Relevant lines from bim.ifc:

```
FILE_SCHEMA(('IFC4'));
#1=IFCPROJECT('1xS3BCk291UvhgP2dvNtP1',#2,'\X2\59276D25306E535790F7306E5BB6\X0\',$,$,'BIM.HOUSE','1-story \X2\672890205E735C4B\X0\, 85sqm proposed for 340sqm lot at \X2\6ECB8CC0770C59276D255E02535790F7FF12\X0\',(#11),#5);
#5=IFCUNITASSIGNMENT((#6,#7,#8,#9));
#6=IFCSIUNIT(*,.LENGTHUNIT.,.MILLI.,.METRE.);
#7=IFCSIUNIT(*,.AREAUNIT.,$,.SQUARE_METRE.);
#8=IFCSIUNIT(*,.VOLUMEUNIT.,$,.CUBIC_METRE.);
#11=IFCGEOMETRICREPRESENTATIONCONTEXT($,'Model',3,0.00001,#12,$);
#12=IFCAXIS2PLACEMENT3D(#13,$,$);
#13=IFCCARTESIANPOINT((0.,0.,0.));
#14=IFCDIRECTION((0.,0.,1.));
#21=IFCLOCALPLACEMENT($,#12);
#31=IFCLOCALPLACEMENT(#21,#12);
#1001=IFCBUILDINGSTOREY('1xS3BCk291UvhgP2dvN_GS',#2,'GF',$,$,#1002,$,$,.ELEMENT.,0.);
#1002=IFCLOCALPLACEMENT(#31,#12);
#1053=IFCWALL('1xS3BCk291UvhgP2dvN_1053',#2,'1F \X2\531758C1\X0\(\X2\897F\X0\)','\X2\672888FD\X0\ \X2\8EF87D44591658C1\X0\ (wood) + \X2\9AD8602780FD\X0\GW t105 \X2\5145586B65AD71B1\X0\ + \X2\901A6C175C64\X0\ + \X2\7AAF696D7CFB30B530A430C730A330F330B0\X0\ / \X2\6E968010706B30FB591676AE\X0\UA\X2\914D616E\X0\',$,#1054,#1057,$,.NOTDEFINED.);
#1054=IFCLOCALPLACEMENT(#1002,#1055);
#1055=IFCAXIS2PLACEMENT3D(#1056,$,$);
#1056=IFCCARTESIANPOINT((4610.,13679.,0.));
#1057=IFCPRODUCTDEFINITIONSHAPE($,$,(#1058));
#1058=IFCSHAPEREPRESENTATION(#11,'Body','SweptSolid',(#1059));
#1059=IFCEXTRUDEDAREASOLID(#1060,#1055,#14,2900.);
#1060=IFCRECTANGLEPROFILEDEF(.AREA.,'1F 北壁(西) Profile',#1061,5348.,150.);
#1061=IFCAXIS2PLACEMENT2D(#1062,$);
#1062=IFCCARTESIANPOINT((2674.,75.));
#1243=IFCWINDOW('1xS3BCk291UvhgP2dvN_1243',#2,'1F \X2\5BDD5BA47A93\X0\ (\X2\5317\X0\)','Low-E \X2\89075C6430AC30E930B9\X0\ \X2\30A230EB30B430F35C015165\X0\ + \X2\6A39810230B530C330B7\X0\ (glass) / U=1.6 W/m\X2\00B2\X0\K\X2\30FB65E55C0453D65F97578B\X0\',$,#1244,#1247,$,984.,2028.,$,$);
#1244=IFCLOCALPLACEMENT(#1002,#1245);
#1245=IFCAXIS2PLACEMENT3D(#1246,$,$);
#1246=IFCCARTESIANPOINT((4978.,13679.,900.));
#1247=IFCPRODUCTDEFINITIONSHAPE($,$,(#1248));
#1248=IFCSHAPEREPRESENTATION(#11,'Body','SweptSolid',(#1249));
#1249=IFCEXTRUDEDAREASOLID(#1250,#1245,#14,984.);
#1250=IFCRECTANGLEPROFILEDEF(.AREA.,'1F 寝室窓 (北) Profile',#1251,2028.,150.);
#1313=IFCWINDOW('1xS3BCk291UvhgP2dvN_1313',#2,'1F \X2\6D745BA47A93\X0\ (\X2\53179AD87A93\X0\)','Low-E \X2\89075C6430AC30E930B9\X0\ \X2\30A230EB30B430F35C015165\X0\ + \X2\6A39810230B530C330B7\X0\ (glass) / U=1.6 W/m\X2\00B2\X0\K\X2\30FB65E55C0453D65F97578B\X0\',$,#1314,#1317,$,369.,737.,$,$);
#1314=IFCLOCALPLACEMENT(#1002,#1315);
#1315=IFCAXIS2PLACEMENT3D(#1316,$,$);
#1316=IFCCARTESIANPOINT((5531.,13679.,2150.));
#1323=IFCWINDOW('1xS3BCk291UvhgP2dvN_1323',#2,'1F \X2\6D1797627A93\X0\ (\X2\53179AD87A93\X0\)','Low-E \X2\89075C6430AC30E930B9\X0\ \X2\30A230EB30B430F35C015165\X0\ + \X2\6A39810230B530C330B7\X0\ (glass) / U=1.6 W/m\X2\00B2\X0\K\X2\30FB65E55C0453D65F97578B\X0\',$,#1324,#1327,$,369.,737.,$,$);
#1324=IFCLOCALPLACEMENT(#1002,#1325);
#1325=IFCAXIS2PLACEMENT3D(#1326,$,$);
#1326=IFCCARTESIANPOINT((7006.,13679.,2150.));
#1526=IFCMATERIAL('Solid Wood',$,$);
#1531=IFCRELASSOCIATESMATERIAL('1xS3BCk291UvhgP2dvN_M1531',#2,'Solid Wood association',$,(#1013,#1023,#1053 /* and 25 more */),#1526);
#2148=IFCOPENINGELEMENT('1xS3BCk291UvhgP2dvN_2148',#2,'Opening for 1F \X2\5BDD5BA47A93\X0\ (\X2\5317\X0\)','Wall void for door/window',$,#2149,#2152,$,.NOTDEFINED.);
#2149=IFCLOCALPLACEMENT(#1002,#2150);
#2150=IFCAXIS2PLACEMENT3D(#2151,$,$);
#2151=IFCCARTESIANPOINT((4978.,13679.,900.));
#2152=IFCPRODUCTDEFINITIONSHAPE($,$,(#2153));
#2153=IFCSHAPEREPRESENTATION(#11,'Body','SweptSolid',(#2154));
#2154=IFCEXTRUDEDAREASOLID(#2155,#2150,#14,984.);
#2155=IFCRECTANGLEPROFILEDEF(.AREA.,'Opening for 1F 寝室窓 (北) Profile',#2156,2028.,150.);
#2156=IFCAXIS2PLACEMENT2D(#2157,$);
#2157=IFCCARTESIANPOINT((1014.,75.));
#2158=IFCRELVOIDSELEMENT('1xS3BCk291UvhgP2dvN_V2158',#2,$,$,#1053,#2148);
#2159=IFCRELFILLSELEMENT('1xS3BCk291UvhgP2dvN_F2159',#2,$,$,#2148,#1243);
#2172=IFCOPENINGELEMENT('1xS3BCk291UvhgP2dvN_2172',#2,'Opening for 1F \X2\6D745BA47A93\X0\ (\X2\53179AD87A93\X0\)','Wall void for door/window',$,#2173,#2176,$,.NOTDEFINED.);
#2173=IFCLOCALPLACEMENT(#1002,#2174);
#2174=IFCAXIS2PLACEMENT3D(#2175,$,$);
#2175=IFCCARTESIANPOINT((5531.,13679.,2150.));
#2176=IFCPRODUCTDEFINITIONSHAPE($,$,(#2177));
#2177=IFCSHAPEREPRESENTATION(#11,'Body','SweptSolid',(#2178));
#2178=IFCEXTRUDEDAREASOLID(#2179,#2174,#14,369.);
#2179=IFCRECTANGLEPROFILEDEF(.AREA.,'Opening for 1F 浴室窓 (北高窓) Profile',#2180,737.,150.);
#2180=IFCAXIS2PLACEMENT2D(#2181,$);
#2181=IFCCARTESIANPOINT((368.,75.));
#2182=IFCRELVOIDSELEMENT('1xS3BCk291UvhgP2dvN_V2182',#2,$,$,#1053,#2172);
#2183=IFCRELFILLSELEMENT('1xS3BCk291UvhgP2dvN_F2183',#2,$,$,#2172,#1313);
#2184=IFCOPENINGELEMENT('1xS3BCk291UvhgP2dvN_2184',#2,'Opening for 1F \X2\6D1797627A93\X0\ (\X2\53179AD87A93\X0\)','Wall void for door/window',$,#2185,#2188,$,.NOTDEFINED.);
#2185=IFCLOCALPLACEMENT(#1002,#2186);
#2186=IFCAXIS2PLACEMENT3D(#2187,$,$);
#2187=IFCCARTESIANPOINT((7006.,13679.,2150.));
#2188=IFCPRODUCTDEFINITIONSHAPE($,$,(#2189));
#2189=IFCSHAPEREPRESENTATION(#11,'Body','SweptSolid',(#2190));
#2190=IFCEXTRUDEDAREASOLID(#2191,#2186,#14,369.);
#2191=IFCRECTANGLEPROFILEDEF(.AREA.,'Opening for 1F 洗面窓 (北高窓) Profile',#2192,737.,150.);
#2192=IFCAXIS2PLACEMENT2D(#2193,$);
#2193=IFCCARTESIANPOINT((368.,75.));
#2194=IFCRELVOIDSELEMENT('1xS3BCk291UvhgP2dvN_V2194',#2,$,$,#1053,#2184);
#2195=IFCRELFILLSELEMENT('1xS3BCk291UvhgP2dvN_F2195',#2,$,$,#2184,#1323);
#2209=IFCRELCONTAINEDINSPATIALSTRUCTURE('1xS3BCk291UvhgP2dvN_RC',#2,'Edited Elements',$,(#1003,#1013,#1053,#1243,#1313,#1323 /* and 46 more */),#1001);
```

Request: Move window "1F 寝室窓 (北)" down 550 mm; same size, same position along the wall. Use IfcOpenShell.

```python
import numpy as np
import ifcopenshell
import ifcopenshell.api.geometry
import ifcopenshell.util.placement
import ifcopenshell.util.unit

model = ifcopenshell.open("bim.ifc")
unit_scale = ifcopenshell.util.unit.calculate_unit_scale(model)

window = model.by_guid("1xS3BCk291UvhgP2dvN_1243")
opening = window.FillsVoids[0].RelatingOpeningElement
dz = -550.0

shift = np.array([0.0, 0.0, dz])
# The window is not placed relative to its opening, so move both.
for product in (opening, window):
    matrix = ifcopenshell.util.placement.get_local_placement(product.ObjectPlacement)
    matrix[:3, 3] += shift
    ifcopenshell.api.geometry.edit_object_placement(model, product=product, matrix=matrix, is_si=False)

print(f"moved by {dz * unit_scale:+.3f} m")

model.write("bim-out.ifc")
```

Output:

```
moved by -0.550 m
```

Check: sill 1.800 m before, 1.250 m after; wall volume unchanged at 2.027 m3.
